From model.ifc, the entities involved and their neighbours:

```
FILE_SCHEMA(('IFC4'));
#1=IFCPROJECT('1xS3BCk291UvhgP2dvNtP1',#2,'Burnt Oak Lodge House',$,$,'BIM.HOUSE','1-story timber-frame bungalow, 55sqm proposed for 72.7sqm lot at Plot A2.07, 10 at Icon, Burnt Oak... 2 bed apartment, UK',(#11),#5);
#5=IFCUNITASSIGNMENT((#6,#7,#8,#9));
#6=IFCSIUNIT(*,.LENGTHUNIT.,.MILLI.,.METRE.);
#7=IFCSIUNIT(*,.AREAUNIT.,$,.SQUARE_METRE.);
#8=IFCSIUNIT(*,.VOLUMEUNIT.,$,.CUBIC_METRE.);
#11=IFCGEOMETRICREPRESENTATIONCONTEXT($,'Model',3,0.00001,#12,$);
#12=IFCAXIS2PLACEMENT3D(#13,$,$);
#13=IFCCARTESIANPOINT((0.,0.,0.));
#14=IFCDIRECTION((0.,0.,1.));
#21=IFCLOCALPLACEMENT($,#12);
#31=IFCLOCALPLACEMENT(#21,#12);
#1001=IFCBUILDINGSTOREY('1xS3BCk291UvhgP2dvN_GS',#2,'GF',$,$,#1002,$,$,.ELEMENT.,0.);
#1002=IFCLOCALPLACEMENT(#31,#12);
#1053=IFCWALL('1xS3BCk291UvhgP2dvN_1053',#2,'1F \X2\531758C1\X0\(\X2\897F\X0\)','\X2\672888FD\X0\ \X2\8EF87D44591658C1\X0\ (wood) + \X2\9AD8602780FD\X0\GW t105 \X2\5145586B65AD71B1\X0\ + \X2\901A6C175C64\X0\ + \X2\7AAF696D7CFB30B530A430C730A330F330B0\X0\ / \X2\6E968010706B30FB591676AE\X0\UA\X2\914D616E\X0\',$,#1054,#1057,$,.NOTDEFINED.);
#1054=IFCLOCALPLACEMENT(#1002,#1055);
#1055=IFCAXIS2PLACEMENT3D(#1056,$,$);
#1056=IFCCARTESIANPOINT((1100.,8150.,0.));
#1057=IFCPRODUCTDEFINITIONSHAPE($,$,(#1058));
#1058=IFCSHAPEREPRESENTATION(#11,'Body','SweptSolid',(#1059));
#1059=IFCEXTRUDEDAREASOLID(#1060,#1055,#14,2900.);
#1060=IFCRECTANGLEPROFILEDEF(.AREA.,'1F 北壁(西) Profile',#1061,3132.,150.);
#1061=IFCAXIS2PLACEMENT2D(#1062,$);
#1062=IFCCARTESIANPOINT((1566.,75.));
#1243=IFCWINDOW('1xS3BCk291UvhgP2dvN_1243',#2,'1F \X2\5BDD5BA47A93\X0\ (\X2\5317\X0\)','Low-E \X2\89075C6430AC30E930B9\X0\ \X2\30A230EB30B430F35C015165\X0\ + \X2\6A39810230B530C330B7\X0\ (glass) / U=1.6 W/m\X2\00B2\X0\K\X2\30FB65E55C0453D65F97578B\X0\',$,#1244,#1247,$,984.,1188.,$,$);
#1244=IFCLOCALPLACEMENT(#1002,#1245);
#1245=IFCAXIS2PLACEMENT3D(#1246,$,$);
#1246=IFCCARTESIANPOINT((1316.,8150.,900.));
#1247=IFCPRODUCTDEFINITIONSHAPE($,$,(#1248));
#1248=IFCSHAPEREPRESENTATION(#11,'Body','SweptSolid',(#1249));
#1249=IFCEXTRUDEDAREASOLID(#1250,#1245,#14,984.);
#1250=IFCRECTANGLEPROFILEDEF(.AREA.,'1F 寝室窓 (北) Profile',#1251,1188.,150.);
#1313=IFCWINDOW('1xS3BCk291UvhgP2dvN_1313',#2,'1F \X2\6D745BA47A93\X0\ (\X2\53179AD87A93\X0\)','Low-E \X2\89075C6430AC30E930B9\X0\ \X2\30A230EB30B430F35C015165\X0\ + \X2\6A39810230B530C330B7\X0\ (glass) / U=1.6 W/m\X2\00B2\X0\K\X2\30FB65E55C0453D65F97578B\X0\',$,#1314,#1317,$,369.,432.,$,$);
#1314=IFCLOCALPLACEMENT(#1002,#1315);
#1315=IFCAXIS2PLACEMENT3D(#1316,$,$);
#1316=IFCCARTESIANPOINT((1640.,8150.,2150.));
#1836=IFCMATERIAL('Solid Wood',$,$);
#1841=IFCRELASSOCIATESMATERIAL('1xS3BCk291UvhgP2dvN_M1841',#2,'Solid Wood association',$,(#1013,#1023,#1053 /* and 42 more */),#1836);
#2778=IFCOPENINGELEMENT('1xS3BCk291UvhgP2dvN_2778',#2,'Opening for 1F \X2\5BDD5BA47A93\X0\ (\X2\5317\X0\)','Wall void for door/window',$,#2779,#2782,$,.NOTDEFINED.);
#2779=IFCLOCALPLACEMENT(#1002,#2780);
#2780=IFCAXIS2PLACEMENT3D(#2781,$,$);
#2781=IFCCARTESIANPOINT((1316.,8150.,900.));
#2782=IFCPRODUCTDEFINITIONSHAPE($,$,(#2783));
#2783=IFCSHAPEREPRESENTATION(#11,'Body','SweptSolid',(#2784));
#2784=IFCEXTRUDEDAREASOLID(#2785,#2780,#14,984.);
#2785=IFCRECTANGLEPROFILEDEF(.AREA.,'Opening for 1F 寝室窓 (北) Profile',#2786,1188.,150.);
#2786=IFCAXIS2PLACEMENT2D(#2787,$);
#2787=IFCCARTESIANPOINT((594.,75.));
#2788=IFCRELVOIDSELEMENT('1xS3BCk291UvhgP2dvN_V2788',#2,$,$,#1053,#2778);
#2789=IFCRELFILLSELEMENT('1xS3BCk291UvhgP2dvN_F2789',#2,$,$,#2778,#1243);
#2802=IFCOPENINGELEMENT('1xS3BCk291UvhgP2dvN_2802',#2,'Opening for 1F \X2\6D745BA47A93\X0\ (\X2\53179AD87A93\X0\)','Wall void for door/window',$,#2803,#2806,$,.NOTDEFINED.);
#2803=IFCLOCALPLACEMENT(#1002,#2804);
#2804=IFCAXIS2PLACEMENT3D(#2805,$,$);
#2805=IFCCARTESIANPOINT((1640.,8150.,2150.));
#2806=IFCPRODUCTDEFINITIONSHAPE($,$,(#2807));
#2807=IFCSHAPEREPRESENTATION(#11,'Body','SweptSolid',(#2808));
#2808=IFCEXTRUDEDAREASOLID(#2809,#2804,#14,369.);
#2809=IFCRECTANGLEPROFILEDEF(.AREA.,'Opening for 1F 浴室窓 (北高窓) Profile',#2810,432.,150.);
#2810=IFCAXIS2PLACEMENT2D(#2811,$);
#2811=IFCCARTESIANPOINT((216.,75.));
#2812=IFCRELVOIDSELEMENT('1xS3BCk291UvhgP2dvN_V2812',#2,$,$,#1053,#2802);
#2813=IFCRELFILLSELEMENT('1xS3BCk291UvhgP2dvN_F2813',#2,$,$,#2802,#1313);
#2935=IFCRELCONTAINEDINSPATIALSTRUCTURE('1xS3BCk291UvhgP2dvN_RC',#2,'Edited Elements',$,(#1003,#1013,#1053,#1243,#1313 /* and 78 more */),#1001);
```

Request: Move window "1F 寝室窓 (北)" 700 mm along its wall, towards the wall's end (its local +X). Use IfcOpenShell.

```python
import ifcopenshell
import ifcopenshell.api.geometry
import ifcopenshell.util.placement

model = ifcopenshell.open("model.ifc")

window = model.by_guid("1xS3BCk291UvhgP2dvN_1243")
opening = window.FillsVoids[0].RelatingOpeningElement
wall = opening.VoidsElements[0].RelatingBuildingElement

wall_matrix = ifcopenshell.util.placement.get_local_placement(wall.ObjectPlacement)
shift = wall_matrix[:3, 0] * 700.0
before = ifcopenshell.util.placement.get_local_placement(window.ObjectPlacement)[:3, 3].copy()

# The window is not placed relative to its opening, so move both.
for product in (opening, window):
    matrix = ifcopenshell.util.placement.get_local_placement(product.ObjectPlacement)
    matrix[:3, 3] += shift
    ifcopenshell.api.geometry.edit_object_placement(model, product=product, matrix=matrix, is_si=False)

after = ifcopenshell.util.placement.get_local_placement(window.ObjectPlacement)[:3, 3]
print("window moved by", (after - before).round(3) + 0.0)

model.write("model_rev.ifc")
```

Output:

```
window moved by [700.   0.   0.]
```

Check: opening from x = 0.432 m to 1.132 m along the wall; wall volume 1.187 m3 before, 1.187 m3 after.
